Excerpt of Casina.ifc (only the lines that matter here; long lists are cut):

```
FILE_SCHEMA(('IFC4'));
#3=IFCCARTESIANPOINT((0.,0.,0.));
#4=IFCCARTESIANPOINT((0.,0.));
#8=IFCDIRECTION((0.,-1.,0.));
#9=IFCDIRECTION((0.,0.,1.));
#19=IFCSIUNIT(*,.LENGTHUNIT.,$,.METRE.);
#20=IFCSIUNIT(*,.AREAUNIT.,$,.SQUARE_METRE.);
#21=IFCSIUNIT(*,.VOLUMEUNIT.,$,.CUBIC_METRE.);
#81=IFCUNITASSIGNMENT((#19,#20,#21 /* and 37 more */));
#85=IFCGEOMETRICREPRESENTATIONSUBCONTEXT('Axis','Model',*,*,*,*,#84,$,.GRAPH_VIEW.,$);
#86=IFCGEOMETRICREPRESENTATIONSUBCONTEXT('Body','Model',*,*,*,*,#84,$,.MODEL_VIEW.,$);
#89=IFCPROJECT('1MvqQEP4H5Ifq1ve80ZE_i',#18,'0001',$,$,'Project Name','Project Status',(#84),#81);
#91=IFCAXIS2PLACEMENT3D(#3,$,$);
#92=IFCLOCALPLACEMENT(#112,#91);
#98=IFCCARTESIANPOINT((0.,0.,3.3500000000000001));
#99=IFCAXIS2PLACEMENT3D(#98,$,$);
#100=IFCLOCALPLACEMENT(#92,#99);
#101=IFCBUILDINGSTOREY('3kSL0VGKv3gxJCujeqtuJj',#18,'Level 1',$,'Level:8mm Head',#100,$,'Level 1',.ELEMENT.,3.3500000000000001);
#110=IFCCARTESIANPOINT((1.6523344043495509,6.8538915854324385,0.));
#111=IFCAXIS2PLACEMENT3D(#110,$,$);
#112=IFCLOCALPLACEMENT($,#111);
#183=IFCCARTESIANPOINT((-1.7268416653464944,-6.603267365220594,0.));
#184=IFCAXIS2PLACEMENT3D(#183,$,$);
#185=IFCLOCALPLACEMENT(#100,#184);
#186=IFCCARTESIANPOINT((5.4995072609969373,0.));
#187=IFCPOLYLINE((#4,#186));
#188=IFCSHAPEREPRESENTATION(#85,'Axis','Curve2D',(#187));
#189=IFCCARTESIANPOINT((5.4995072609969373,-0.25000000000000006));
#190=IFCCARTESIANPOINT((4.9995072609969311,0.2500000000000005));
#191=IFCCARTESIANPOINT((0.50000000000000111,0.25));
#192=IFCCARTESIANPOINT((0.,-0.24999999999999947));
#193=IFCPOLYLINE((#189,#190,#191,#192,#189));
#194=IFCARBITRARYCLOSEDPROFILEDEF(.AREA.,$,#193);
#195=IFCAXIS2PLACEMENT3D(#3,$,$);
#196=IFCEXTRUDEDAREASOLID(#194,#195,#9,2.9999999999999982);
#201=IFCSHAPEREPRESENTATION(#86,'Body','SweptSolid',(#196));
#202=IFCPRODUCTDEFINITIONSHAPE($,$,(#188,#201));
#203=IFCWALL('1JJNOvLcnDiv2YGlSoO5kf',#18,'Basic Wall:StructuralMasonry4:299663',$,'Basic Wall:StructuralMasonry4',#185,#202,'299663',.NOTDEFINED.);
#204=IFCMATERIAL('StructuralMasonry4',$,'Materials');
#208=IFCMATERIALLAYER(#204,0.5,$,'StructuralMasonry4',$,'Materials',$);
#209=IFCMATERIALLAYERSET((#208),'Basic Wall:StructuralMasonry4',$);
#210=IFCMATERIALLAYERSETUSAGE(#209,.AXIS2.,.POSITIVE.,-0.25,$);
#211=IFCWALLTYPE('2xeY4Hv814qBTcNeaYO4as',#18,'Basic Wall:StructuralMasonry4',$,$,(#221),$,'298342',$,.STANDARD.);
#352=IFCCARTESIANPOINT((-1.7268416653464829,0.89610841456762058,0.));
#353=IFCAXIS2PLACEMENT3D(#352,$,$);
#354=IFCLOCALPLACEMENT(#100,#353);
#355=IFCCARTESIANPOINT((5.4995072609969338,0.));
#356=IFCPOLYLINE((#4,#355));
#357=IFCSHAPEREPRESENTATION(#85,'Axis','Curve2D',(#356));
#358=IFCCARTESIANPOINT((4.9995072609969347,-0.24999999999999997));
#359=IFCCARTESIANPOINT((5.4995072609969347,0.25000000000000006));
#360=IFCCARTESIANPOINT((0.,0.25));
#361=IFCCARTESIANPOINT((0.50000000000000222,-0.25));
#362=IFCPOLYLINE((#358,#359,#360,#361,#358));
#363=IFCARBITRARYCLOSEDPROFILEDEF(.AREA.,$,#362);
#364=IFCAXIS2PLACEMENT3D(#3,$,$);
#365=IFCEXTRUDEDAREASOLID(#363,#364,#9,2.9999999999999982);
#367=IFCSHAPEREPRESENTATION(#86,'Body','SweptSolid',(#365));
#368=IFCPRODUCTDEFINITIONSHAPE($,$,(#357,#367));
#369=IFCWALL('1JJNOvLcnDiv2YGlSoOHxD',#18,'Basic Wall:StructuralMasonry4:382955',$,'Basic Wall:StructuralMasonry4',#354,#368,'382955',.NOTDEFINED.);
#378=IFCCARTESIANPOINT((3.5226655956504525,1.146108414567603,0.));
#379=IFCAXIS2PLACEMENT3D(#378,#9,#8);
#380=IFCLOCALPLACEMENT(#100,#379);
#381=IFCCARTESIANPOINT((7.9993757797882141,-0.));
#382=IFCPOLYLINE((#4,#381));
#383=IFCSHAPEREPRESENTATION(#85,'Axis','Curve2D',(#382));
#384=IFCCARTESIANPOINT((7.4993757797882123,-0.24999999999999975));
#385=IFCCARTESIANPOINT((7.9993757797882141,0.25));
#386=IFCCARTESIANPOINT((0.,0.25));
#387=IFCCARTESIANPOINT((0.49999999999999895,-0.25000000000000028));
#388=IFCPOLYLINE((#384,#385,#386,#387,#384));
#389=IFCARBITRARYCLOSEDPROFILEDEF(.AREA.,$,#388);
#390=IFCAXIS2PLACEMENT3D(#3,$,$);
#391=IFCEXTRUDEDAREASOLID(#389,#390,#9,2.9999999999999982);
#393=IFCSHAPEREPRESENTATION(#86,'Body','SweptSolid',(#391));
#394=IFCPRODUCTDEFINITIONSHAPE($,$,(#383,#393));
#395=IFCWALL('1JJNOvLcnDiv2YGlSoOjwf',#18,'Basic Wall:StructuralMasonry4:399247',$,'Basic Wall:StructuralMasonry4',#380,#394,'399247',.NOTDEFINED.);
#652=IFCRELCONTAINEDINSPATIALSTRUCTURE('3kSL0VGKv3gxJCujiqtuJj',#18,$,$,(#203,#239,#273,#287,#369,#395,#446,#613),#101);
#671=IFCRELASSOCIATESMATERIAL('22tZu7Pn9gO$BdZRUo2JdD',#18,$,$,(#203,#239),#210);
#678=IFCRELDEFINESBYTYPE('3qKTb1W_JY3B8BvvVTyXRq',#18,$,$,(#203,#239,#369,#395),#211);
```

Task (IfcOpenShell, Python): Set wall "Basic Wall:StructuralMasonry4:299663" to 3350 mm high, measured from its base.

```python
import ifcopenshell
import ifcopenshell.geom
import ifcopenshell.util.representation
import ifcopenshell.util.shape

model = ifcopenshell.open("Casina.ifc")
settings = ifcopenshell.geom.settings()


def volume(element):
    """Net volume in cubic metres, openings subtracted."""
    shape = ifcopenshell.geom.create_shape(settings, element)
    return ifcopenshell.util.shape.get_volume(shape.geometry)


wall = model.by_guid("1JJNOvLcnDiv2YGlSoO5kf")
before = volume(wall)

body = ifcopenshell.util.representation.get_representation(wall, "Model", "Body")
solid = body.Items[0]
old_height = solid.Depth
solid.Depth = 3.35
after = volume(wall)

print(f"height {old_height:g} -> {solid.Depth:g}, volume {before:.3f} -> {after:.3f} m3")

model.write("Casina_v2.ifc")
```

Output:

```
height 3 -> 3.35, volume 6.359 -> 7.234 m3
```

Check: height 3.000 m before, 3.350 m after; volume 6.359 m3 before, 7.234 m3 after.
